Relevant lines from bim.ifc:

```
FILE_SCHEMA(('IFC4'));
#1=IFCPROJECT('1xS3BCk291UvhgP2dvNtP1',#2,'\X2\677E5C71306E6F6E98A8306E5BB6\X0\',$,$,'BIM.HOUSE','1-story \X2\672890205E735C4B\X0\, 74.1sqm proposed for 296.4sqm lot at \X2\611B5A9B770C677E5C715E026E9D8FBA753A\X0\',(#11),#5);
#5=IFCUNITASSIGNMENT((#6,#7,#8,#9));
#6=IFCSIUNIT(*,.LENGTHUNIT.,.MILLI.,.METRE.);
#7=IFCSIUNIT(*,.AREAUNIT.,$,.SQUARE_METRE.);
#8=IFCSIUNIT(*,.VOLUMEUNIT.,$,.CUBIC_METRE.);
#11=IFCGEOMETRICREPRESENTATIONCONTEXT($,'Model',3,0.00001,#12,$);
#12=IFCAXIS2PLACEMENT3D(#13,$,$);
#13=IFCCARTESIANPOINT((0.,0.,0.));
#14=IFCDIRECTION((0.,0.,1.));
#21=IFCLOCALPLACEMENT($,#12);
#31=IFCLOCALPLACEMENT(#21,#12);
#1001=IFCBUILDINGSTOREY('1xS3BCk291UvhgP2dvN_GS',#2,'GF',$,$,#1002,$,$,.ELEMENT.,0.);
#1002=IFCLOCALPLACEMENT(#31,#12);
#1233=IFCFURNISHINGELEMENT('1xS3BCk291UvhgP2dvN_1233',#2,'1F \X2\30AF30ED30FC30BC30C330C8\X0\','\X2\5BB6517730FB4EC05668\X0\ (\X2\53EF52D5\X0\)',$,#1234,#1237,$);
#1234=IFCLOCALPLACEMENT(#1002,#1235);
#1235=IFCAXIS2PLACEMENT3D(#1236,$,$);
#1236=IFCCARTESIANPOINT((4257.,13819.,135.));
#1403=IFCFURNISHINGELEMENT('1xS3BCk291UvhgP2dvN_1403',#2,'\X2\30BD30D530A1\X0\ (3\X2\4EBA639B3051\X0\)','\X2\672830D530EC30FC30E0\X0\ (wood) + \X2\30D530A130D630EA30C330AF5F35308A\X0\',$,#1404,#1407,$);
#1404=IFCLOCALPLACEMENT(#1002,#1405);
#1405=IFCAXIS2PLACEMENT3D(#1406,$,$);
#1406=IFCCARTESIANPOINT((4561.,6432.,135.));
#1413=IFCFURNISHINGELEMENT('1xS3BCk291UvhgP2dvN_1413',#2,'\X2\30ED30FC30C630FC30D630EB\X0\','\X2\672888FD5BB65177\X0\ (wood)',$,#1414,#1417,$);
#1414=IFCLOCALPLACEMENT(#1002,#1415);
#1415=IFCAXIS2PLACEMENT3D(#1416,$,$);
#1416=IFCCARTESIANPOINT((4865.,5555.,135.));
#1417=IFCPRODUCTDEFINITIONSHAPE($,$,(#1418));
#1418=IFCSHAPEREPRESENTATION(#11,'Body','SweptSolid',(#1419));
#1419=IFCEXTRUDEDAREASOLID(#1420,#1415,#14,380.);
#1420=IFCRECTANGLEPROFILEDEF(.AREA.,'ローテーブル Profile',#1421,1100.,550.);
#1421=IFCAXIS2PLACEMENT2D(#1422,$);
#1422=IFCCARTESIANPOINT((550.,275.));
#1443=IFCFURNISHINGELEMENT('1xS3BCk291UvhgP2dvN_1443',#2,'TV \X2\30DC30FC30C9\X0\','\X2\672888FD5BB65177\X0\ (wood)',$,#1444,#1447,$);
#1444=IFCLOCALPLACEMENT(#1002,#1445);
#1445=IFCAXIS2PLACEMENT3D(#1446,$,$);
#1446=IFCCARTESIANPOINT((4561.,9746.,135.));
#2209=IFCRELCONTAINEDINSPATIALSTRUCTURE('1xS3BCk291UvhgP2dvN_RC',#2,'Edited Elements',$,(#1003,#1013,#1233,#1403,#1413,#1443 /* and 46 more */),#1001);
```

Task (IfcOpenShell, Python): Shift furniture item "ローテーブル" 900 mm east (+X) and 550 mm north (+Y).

```python
import ifcopenshell
import ifcopenshell.api.geometry
import ifcopenshell.util.placement
import ifcopenshell.util.unit

model = ifcopenshell.open("bim.ifc")
unit_scale = ifcopenshell.util.unit.calculate_unit_scale(model)

item = model.by_guid("1xS3BCk291UvhgP2dvN_1413")
matrix = ifcopenshell.util.placement.get_local_placement(item.ObjectPlacement)
matrix[0, 3] += 0.9 / unit_scale
matrix[1, 3] += 0.55 / unit_scale
ifcopenshell.api.geometry.edit_object_placement(model, product=item, matrix=matrix, is_si=False)

print(ifcopenshell.util.placement.get_local_placement(item.ObjectPlacement).round(3) + 0.0)

model.write("bim_v2.ifc")
```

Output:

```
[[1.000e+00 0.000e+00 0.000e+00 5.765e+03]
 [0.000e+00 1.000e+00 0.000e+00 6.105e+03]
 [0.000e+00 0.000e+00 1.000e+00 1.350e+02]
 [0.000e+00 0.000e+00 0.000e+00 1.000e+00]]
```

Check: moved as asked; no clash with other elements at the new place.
